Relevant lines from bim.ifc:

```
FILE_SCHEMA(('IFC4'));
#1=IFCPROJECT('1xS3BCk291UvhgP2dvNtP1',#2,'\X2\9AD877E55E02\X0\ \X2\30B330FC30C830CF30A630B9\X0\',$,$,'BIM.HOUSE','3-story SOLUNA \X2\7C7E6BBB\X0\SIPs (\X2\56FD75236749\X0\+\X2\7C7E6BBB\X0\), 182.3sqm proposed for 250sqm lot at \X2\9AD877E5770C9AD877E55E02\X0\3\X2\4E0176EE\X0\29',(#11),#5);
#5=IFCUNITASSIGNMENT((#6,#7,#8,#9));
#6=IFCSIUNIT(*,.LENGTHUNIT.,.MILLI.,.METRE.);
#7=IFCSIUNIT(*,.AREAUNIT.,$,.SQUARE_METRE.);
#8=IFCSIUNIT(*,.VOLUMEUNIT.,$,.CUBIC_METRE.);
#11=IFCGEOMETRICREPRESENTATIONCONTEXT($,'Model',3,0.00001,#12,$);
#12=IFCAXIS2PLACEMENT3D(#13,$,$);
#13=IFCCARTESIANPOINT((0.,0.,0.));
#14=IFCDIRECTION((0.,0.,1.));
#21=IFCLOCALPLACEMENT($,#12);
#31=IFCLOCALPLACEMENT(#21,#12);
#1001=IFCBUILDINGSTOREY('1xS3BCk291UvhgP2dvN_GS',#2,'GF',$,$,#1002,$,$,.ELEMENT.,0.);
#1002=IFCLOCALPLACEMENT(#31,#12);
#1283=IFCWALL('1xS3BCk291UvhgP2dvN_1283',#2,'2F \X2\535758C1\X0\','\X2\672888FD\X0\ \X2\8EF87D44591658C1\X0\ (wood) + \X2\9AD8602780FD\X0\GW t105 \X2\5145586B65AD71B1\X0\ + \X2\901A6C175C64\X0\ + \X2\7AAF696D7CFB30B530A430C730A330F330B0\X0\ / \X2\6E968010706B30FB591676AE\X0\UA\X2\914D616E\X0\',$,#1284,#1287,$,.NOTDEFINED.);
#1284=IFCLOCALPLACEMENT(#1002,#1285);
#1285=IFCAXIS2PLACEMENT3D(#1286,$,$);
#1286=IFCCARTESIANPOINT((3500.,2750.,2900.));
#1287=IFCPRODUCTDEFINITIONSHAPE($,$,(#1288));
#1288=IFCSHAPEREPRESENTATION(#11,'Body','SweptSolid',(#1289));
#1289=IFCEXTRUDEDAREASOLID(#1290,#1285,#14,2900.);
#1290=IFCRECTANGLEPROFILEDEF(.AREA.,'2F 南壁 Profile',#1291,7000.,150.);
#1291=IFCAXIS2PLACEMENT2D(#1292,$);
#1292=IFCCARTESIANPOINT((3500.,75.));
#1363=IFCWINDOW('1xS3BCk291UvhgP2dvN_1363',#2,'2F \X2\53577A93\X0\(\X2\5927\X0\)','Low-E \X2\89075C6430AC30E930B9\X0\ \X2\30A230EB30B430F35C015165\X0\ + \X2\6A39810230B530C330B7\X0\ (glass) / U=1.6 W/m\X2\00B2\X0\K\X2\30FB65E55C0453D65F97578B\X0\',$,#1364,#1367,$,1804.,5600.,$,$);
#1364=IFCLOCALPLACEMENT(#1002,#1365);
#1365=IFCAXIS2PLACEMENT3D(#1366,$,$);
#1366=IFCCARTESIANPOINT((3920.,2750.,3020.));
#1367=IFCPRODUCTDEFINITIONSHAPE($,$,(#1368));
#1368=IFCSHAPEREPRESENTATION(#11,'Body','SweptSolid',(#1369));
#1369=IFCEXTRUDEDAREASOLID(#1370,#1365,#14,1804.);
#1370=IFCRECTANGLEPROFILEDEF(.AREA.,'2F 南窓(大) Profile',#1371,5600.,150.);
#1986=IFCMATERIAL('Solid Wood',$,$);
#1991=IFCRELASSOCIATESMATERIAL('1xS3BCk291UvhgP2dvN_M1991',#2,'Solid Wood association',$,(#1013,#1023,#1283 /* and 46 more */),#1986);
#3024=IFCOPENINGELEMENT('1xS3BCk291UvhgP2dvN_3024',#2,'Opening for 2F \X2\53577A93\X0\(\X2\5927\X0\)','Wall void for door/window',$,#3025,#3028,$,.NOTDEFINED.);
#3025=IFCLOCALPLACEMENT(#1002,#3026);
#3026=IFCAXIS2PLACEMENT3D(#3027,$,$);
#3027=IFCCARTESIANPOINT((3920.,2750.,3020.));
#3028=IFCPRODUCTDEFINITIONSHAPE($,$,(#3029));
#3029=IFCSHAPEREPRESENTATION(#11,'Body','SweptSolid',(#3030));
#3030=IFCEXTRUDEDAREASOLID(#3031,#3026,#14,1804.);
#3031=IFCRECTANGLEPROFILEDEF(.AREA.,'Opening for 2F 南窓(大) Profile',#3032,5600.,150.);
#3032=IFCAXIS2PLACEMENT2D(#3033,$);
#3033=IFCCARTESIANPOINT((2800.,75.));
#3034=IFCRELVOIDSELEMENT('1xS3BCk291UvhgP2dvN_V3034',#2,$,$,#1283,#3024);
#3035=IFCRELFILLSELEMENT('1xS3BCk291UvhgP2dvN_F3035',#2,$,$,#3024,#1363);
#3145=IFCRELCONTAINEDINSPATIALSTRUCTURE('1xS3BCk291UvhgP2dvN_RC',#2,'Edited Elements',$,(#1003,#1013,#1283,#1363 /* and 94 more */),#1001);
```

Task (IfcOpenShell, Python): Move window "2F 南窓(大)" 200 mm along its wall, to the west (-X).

```python
import ifcopenshell
import ifcopenshell.api.geometry
import ifcopenshell.util.placement
import ifcopenshell.util.unit

model = ifcopenshell.open("bim.ifc")
unit_scale = ifcopenshell.util.unit.calculate_unit_scale(model)

window = model.by_guid("1xS3BCk291UvhgP2dvN_1363")
opening = window.FillsVoids[0].RelatingOpeningElement
wall = opening.VoidsElements[0].RelatingBuildingElement

wall_matrix = ifcopenshell.util.placement.get_local_placement(wall.ObjectPlacement)
shift = wall_matrix[:3, 0] * -0.2 / unit_scale
before = ifcopenshell.util.placement.get_local_placement(window.ObjectPlacement)[:3, 3].copy()

# The window is not placed relative to its opening, so move both.
for product in (opening, window):
    matrix = ifcopenshell.util.placement.get_local_placement(product.ObjectPlacement)
    matrix[:3, 3] += shift
    ifcopenshell.api.geometry.edit_object_placement(model, product=product, matrix=matrix, is_si=False)

after = ifcopenshell.util.placement.get_local_placement(window.ObjectPlacement)[:3, 3]
print("window moved by", (after - before).round(3) + 0.0)

model.write("bim_edited.ifc")
```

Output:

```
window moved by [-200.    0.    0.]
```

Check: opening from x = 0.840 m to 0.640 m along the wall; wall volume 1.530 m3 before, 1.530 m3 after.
